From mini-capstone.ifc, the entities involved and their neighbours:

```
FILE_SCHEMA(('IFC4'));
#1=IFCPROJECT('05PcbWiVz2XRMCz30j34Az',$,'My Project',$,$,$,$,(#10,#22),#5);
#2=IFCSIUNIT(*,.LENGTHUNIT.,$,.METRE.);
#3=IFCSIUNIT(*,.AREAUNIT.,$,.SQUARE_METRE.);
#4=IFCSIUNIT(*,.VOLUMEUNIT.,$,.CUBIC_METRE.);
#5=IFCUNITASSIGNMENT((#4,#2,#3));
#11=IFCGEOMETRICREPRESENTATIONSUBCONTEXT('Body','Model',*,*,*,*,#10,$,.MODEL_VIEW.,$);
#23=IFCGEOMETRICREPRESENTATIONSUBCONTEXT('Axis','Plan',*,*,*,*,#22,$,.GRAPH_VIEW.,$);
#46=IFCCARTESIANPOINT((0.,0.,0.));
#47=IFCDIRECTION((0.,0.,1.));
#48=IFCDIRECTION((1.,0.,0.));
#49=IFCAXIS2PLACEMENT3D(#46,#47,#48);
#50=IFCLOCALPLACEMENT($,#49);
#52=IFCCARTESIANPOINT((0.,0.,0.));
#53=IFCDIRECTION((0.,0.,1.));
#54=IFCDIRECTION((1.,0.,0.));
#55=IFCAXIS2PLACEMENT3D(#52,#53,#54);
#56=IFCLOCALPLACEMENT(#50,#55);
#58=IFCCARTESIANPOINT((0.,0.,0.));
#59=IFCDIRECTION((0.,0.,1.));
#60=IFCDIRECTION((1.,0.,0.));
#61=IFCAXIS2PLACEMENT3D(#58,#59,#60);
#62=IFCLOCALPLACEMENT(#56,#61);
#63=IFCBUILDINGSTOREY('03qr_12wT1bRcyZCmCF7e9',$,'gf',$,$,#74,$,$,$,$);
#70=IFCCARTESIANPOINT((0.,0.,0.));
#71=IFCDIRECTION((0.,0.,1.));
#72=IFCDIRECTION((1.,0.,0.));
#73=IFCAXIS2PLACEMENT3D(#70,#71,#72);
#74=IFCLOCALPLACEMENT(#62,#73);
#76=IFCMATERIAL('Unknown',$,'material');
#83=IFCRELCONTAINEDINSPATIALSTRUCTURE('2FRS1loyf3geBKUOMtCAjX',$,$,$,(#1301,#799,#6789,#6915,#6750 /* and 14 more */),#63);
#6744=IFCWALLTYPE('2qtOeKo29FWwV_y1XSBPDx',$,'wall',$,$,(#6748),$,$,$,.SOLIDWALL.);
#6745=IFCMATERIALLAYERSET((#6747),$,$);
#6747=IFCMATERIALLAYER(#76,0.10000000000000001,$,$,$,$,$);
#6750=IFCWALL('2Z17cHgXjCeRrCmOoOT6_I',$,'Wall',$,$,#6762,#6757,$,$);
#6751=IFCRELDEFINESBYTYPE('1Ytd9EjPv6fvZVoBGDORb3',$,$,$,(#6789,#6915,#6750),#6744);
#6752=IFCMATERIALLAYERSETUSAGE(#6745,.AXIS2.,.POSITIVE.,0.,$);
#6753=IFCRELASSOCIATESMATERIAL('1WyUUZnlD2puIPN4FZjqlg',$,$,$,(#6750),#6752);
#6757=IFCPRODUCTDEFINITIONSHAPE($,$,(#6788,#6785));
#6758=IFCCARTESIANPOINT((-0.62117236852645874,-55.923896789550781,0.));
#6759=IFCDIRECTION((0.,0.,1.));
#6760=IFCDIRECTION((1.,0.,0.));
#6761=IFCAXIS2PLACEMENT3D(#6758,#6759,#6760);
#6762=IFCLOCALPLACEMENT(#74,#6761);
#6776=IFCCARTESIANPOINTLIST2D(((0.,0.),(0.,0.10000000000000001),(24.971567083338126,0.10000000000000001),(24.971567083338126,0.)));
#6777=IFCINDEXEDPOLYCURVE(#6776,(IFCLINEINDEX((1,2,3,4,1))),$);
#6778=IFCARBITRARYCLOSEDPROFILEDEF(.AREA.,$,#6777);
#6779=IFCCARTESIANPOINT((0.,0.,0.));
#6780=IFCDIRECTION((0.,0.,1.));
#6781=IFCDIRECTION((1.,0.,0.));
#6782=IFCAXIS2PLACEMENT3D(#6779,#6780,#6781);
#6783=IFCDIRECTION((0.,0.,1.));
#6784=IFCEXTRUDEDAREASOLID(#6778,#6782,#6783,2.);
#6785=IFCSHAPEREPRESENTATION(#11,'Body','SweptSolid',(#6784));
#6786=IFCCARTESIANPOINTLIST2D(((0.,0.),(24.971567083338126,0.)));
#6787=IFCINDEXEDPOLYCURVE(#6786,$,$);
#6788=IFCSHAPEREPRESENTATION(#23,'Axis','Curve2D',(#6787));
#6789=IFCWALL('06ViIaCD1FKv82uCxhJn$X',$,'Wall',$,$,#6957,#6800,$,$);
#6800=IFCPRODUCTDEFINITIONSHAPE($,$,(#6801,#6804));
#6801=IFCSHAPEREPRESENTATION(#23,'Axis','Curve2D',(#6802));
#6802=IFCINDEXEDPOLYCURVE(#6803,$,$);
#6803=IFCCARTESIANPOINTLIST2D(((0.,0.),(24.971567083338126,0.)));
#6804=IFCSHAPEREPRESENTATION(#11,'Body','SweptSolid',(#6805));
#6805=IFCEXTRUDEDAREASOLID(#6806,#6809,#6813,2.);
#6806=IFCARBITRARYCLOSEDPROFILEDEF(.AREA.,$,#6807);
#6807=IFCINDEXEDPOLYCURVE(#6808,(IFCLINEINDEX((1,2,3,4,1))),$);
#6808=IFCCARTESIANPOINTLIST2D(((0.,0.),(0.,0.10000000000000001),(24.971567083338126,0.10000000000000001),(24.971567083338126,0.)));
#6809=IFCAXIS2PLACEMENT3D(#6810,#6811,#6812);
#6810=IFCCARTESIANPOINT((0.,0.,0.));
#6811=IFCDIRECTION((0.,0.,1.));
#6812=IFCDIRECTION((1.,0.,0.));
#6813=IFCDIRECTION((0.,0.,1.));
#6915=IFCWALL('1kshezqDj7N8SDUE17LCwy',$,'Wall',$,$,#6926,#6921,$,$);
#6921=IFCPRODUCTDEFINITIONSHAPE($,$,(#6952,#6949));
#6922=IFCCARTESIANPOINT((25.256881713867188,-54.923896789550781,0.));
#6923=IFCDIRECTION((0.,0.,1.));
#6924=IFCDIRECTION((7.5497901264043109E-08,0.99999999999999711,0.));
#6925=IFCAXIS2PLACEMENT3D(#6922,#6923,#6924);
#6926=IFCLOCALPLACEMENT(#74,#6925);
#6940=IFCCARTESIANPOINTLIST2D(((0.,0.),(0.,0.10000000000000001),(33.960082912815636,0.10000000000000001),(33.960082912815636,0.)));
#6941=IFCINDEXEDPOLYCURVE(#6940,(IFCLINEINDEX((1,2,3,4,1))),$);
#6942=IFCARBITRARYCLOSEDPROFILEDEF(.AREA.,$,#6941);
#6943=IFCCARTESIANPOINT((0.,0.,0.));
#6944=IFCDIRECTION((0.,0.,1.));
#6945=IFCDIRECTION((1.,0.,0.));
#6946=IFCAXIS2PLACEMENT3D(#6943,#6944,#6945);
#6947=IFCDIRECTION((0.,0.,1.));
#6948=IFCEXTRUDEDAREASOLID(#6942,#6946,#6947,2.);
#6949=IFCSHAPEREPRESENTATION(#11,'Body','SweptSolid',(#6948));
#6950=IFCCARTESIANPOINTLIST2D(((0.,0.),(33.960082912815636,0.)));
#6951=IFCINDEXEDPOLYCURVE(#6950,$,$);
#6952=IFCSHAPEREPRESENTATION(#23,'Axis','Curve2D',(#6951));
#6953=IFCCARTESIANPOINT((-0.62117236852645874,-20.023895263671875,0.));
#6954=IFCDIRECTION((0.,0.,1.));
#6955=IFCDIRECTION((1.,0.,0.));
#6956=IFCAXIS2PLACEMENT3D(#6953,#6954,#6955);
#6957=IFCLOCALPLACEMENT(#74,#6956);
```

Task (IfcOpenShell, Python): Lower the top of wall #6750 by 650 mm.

```python
import ifcopenshell
import ifcopenshell.geom
import ifcopenshell.util.representation
import ifcopenshell.util.shape
import ifcopenshell.util.unit

model = ifcopenshell.open("mini-capstone.ifc")
unit_scale = ifcopenshell.util.unit.calculate_unit_scale(model)
settings = ifcopenshell.geom.settings()


def volume(element):
    """Net volume in cubic metres, openings subtracted."""
    shape = ifcopenshell.geom.create_shape(settings, element)
    return ifcopenshell.util.shape.get_volume(shape.geometry)


wall = model.by_guid("2Z17cHgXjCeRrCmOoOT6_I")
before = volume(wall)

body = ifcopenshell.util.representation.get_representation(wall, "Model", "Body")
solid = body.Items[0]
old_height = solid.Depth
solid.Depth -= 0.65 / unit_scale
after = volume(wall)

print(f"height {old_height:g} -> {solid.Depth:g}, volume {before:.3f} -> {after:.3f} m3")

model.write("mini-capstone_v2.ifc")
```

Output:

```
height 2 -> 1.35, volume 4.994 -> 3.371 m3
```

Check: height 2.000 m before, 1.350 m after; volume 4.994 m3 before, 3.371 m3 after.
